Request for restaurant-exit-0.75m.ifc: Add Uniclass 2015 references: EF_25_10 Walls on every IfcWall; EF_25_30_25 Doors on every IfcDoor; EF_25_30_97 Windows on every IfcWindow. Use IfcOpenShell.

First a look at what the model holds.

```python
import ifcopenshell

model = ifcopenshell.open("restaurant-exit-0.75m.ifc")
print(model.schema)
print("classifications:", [c.Name for c in model.by_type("IfcClassification")])
for ifc_class in ("IfcDoor", "IfcRoof", "IfcStair", "IfcWall", "IfcWindow"):
    print(ifc_class, len(model.by_type(ifc_class)))
```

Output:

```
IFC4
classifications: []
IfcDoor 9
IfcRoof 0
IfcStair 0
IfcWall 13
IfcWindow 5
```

```python
import ifcopenshell
import ifcopenshell.api.classification

model = ifcopenshell.open("restaurant-exit-0.75m.ifc")

system = ifcopenshell.api.classification.add_classification(model, classification="Uniclass 2015")

codes = {
    "IfcWall": ("EF_25_10", "Walls"),
    "IfcDoor": ("EF_25_30_25", "Doors"),
    "IfcWindow": ("EF_25_30_97", "Windows"),
}
for ifc_class, (code, name) in codes.items():
    products = model.by_type(ifc_class)
    ifcopenshell.api.classification.add_reference(
        model, products=products, classification=system, identification=code, name=name
    )
    print(code, len(products))

model.write("restaurant-exit-0.75m_updated.ifc")
```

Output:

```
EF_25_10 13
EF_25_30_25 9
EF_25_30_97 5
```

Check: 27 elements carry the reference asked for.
